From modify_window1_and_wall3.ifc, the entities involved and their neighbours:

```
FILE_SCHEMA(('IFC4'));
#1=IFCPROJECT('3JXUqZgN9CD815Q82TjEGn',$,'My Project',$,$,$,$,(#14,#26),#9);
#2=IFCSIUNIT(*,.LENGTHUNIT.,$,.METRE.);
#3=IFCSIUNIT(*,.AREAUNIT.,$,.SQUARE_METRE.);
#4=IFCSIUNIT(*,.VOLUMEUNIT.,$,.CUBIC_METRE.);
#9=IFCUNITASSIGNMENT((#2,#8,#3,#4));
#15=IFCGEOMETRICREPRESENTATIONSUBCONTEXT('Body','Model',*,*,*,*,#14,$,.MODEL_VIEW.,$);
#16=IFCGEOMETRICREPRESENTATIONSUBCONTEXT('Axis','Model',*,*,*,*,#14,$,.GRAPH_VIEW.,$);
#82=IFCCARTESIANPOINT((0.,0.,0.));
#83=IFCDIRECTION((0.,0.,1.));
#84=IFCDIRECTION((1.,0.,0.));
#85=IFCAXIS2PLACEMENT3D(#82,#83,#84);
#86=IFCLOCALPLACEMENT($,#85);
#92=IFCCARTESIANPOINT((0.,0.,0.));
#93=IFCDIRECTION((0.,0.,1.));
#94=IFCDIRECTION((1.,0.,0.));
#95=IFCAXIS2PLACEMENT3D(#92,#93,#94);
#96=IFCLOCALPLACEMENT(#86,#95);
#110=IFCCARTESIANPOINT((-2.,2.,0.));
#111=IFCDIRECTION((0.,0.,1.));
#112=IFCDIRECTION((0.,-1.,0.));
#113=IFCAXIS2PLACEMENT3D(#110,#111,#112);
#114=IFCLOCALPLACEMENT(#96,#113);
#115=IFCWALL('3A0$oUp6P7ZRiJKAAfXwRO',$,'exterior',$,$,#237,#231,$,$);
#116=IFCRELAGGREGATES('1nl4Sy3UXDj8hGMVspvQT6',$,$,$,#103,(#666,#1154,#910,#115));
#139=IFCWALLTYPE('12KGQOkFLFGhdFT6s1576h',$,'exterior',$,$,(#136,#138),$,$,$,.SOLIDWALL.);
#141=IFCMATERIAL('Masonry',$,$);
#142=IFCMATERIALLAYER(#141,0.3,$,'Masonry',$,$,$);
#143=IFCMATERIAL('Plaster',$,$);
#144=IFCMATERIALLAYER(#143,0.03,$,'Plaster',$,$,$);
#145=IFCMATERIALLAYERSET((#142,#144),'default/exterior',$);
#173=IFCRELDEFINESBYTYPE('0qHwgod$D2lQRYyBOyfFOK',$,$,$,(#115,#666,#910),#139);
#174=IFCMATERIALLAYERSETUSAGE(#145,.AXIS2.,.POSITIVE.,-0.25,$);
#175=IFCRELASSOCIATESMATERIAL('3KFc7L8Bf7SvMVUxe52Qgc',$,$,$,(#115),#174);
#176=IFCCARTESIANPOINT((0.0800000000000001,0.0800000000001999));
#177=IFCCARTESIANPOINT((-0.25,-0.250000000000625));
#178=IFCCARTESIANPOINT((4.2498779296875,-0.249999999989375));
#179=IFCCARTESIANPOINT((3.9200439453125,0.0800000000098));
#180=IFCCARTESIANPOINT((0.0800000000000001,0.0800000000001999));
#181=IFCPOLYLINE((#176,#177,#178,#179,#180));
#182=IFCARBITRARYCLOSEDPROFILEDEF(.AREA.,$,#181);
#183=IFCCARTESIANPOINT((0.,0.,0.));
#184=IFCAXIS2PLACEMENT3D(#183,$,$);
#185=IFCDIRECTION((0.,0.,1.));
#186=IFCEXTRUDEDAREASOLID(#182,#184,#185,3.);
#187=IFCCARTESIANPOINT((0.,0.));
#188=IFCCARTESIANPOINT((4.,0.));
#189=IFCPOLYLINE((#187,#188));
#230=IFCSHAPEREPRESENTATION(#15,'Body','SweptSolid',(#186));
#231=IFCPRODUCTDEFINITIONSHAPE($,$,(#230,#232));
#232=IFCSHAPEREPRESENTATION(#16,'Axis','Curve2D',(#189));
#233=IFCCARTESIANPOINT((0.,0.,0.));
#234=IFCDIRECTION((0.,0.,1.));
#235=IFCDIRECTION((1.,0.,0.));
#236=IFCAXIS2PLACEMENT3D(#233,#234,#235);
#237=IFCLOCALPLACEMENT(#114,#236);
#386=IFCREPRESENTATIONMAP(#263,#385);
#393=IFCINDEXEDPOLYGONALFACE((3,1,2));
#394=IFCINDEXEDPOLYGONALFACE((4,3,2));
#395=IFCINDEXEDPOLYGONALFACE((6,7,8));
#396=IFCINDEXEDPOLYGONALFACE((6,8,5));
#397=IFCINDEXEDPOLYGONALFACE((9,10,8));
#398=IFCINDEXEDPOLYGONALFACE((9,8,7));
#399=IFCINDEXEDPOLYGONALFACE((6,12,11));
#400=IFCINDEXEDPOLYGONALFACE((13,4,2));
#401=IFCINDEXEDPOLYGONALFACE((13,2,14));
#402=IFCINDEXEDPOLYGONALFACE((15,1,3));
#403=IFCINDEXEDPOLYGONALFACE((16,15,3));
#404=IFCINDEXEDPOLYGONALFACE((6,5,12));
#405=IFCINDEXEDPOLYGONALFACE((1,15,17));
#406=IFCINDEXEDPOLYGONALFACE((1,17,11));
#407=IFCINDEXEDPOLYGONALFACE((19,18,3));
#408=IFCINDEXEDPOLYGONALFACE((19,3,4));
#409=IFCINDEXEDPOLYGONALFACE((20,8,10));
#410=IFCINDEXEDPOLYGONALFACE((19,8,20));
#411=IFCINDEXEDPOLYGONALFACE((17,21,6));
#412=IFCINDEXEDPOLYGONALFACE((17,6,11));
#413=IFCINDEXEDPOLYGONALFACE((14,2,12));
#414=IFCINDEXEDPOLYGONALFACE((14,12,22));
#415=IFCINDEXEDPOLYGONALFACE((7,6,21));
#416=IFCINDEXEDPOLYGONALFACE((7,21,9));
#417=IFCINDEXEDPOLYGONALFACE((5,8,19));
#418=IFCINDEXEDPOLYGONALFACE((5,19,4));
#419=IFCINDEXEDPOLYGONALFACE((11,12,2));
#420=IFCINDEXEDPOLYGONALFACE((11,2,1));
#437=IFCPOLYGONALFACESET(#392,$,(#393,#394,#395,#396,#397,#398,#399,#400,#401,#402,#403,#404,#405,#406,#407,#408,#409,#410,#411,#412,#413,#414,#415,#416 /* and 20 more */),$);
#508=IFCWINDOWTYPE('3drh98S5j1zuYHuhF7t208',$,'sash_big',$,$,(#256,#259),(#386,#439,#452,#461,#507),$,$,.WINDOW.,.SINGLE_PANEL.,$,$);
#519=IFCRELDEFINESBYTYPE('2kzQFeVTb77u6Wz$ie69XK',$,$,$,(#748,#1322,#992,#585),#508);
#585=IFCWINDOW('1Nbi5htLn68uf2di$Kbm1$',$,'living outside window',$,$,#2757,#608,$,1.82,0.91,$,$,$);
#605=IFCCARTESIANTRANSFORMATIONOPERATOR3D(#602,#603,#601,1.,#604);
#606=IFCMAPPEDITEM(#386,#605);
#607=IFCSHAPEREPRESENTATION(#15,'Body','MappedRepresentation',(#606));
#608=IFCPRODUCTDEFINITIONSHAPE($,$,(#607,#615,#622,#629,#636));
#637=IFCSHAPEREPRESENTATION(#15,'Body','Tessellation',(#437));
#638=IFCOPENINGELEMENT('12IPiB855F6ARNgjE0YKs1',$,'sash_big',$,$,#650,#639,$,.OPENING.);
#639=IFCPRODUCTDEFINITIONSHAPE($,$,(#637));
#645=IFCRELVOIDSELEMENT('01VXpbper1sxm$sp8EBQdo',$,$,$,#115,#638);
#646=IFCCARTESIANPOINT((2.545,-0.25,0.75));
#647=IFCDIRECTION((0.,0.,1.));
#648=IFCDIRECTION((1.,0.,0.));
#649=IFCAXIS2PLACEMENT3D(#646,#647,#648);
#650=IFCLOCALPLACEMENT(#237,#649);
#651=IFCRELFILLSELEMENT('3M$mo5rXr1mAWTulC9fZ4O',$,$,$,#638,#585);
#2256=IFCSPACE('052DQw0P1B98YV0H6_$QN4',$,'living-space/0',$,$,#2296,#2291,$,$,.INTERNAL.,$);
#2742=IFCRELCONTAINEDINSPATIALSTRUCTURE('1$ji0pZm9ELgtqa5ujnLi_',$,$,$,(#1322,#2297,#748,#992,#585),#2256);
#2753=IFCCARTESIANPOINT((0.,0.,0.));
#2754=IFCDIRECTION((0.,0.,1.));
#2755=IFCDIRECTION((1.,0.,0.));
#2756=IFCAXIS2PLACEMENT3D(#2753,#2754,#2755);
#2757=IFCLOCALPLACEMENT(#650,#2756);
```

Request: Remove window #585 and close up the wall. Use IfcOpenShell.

```python
import ifcopenshell
import ifcopenshell.api.feature
import ifcopenshell.api.root
import ifcopenshell.geom
import ifcopenshell.util.shape

model = ifcopenshell.open("modify_window1_and_wall3.ifc")
settings = ifcopenshell.geom.settings()


def volume(element):
    """Net volume in cubic metres, openings subtracted."""
    shape = ifcopenshell.geom.create_shape(settings, element)
    return ifcopenshell.util.shape.get_volume(shape.geometry)


window = model.by_id(585)
opening = window.FillsVoids[0].RelatingOpeningElement
wall = opening.VoidsElements[0].RelatingBuildingElement
before = volume(wall)

ifcopenshell.api.root.remove_product(model, product=window)
ifcopenshell.api.feature.remove_feature(model, feature=opening)

after = volume(wall)

print(f"wall volume {before:.3f} -> {after:.3f} m3")

model.write("modify_window1_and_wall3_v2.ifc")
```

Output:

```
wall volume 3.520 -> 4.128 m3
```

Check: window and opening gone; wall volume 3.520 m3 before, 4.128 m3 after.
